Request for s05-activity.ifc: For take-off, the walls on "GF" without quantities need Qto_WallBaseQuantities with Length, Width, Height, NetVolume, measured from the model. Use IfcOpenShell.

First a look at what the model holds.

```python
import ifcopenshell
import ifcopenshell.util.element
import ifcopenshell.util.unit

model = ifcopenshell.open("s05-activity.ifc")
print(model.schema)
for unit_type in ("LENGTHUNIT", "AREAUNIT", "VOLUMEUNIT"):
    print(unit_type, ifcopenshell.util.unit.calculate_unit_scale(model, unit_type))
storey = next(s for s in model.by_type("IfcBuildingStorey") if s.Name == "GF")
walls = [e for e in ifcopenshell.util.element.get_decomposition(storey) if e.is_a("IfcWall")]
for e in sorted(walls, key=lambda e: e.id()):
    print(e.id(), e.is_a(), e.Name, list(ifcopenshell.util.element.get_psets(e, qtos_only=True)), sep=" | ")
```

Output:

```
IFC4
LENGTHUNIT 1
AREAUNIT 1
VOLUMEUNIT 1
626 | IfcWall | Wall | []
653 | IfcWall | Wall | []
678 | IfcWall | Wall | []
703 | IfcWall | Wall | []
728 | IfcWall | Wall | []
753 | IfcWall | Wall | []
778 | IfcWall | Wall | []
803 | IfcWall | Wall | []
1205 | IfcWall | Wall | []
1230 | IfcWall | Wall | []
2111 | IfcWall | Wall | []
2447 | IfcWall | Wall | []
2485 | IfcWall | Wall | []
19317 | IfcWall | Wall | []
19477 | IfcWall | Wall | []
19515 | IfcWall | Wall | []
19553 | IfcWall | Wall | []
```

```python
import ifcopenshell
import ifcopenshell.api.pset
import ifcopenshell.geom
import ifcopenshell.util.element
import ifcopenshell.util.shape
import ifcopenshell.util.unit

model = ifcopenshell.open("s05-activity.ifc")
unit_scale = ifcopenshell.util.unit.calculate_unit_scale(model)
volume_scale = ifcopenshell.util.unit.calculate_unit_scale(model, "VOLUMEUNIT")
settings = ifcopenshell.geom.settings()

storey = next(s for s in model.by_type("IfcBuildingStorey") if s.Name == "GF")
walls = [e for e in ifcopenshell.util.element.get_decomposition(storey) if e.is_a("IfcWall")]

for e in sorted(walls, key=lambda e: e.id()):
    if ifcopenshell.util.element.get_psets(e, qtos_only=True, should_inherit=False):
        continue
    # Geometry comes back in metres, in the element's own axes.
    shape = ifcopenshell.geom.create_shape(settings, e)
    values = {
        "Length": ifcopenshell.util.shape.get_x(shape.geometry) / unit_scale,
        "Width": ifcopenshell.util.shape.get_y(shape.geometry) / unit_scale,
        "Height": ifcopenshell.util.shape.get_z(shape.geometry) / unit_scale,
        "NetVolume": ifcopenshell.util.shape.get_volume(shape.geometry) / volume_scale,
    }
    qto = ifcopenshell.api.pset.add_qto(model, product=e, name="Qto_WallBaseQuantities")
    ifcopenshell.api.pset.edit_qto(model, qto=qto, properties=values)
    print(e.id(), {k: round(v, 3) for k, v in values.items()})

model.write("s05-activity_rev.ifc")
```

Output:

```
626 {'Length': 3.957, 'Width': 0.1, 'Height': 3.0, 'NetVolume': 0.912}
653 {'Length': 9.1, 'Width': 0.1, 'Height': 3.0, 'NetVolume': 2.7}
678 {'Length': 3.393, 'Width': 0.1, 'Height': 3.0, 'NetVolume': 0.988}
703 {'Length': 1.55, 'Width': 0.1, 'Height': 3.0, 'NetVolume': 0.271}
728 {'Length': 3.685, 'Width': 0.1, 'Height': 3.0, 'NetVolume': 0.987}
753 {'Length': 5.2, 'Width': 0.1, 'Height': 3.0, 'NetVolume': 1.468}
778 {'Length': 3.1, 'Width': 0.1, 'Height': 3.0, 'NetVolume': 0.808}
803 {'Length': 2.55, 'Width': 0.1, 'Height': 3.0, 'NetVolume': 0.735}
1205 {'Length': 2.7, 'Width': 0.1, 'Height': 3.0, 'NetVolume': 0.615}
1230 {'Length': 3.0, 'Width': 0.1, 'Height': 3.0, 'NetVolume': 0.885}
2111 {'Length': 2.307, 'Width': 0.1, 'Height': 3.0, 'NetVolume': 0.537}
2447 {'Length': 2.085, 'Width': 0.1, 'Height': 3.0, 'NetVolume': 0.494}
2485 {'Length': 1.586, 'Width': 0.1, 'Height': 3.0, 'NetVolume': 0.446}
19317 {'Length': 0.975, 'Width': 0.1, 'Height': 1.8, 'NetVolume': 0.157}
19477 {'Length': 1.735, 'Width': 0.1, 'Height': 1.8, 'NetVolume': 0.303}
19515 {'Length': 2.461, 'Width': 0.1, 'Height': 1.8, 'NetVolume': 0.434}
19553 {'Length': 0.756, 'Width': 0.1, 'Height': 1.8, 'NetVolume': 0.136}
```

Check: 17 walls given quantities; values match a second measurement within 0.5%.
